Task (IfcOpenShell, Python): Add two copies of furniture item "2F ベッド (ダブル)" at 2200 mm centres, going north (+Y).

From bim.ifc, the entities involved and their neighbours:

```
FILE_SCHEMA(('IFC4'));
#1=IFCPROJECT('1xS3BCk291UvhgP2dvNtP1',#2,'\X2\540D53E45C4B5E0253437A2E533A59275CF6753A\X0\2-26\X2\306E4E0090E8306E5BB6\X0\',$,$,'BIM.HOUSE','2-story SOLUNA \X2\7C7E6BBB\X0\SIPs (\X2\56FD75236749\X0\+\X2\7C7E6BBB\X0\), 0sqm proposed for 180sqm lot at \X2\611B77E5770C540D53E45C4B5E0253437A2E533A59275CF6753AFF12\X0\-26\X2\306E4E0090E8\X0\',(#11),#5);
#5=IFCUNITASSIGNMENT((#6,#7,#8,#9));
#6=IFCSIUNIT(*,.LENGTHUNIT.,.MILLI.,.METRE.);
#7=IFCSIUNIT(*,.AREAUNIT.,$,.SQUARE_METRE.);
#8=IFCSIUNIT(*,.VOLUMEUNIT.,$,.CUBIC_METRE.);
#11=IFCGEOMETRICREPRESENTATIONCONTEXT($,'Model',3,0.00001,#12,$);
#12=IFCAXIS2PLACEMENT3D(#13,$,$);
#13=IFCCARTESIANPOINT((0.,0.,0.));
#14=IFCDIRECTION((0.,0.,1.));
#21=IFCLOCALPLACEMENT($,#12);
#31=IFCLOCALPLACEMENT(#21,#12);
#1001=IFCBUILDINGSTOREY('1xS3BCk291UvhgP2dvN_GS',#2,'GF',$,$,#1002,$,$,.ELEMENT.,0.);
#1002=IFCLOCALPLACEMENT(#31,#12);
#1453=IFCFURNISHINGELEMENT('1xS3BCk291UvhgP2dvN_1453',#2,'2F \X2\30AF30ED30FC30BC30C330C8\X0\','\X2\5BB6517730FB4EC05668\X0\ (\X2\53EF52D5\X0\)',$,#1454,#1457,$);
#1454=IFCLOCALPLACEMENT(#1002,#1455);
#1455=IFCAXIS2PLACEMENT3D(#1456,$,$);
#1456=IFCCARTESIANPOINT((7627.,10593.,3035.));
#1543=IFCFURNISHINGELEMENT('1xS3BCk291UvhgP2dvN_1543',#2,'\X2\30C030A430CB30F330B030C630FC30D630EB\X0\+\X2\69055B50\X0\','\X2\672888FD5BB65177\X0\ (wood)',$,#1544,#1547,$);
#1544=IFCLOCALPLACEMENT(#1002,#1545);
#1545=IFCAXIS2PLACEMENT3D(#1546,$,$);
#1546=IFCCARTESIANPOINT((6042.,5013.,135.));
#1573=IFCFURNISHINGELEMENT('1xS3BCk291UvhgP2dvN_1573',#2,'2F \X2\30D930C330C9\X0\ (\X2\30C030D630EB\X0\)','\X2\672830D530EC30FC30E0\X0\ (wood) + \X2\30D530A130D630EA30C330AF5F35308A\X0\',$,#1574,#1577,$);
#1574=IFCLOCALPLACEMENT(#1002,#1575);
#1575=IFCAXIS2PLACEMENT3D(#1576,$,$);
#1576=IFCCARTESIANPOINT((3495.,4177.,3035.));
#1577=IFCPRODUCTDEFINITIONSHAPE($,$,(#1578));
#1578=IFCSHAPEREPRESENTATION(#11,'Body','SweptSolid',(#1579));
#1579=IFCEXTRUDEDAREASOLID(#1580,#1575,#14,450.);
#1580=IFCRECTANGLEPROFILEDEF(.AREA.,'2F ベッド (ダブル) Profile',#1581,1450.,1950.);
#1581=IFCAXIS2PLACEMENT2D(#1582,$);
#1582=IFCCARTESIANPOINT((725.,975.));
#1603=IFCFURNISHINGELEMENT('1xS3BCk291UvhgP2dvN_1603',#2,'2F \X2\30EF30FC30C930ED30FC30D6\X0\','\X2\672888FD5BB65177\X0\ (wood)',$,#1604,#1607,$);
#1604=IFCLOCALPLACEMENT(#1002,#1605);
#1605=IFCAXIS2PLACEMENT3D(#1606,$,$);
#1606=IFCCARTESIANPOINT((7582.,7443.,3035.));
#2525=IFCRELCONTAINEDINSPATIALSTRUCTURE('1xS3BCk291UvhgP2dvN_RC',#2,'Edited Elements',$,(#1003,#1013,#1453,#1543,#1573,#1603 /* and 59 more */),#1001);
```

```python
import numpy as np
import ifcopenshell
import ifcopenshell.api.geometry
import ifcopenshell.api.root
import ifcopenshell.util.element
import ifcopenshell.util.placement

model = ifcopenshell.open("bim.ifc")


def reuse_history(source, copy):
    """copy_class also copies each property set's owner history, people and application; keep the originals."""
    for rel in copy.IsDefinedBy:
        if rel.is_a("IfcRelDefinesByProperties") and (history := rel.RelatingPropertyDefinition.OwnerHistory):
            rel.RelatingPropertyDefinition.OwnerHistory = source.OwnerHistory
            ifcopenshell.util.element.remove_deep2(model, history)


source = model.by_guid("1xS3BCk291UvhgP2dvN_1573")
base = ifcopenshell.util.placement.get_local_placement(source.ObjectPlacement)
step = np.array([0.0, 1.0, 0.0]) * 2200.0

for i in range(1, 3):
    copy = ifcopenshell.api.root.copy_class(model, product=source)
    copy.Representation = ifcopenshell.util.element.copy_deep(
        model, source.Representation, exclude=["IfcGeometricRepresentationContext", "IfcRepresentationMap"]
    )
    reuse_history(source, copy)
    matrix = base.copy()
    matrix[:3, 3] += i * step
    print("added at", matrix[:3, 3].round(3) + 0.0)
    ifcopenshell.api.geometry.edit_object_placement(model, product=copy, matrix=matrix, is_si=False)

model.write("bim_rev.ifc")
```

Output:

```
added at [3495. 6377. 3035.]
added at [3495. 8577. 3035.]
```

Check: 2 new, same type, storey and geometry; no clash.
